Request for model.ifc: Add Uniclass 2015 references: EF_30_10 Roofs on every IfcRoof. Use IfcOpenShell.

First a look at what the model holds.

```python
import ifcopenshell

model = ifcopenshell.open("model.ifc")
print(model.schema)
print("classifications:", [c.Name for c in model.by_type("IfcClassification")])
for ifc_class in ("IfcDoor", "IfcRoof", "IfcStair", "IfcWall", "IfcWindow"):
    print(ifc_class, len(model.by_type(ifc_class)))
```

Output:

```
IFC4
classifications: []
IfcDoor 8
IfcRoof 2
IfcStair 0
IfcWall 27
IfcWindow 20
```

```python
import ifcopenshell
import ifcopenshell.api.classification

model = ifcopenshell.open("model.ifc")

system = ifcopenshell.api.classification.add_classification(model, classification="Uniclass 2015")

codes = {
    "IfcRoof": ("EF_30_10", "Roofs"),
}
for ifc_class, (code, name) in codes.items():
    products = model.by_type(ifc_class)
    ifcopenshell.api.classification.add_reference(
        model, products=products, classification=system, identification=code, name=name
    )
    print(code, len(products))

model.write("model_updated.ifc")
```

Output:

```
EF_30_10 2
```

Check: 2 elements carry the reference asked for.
